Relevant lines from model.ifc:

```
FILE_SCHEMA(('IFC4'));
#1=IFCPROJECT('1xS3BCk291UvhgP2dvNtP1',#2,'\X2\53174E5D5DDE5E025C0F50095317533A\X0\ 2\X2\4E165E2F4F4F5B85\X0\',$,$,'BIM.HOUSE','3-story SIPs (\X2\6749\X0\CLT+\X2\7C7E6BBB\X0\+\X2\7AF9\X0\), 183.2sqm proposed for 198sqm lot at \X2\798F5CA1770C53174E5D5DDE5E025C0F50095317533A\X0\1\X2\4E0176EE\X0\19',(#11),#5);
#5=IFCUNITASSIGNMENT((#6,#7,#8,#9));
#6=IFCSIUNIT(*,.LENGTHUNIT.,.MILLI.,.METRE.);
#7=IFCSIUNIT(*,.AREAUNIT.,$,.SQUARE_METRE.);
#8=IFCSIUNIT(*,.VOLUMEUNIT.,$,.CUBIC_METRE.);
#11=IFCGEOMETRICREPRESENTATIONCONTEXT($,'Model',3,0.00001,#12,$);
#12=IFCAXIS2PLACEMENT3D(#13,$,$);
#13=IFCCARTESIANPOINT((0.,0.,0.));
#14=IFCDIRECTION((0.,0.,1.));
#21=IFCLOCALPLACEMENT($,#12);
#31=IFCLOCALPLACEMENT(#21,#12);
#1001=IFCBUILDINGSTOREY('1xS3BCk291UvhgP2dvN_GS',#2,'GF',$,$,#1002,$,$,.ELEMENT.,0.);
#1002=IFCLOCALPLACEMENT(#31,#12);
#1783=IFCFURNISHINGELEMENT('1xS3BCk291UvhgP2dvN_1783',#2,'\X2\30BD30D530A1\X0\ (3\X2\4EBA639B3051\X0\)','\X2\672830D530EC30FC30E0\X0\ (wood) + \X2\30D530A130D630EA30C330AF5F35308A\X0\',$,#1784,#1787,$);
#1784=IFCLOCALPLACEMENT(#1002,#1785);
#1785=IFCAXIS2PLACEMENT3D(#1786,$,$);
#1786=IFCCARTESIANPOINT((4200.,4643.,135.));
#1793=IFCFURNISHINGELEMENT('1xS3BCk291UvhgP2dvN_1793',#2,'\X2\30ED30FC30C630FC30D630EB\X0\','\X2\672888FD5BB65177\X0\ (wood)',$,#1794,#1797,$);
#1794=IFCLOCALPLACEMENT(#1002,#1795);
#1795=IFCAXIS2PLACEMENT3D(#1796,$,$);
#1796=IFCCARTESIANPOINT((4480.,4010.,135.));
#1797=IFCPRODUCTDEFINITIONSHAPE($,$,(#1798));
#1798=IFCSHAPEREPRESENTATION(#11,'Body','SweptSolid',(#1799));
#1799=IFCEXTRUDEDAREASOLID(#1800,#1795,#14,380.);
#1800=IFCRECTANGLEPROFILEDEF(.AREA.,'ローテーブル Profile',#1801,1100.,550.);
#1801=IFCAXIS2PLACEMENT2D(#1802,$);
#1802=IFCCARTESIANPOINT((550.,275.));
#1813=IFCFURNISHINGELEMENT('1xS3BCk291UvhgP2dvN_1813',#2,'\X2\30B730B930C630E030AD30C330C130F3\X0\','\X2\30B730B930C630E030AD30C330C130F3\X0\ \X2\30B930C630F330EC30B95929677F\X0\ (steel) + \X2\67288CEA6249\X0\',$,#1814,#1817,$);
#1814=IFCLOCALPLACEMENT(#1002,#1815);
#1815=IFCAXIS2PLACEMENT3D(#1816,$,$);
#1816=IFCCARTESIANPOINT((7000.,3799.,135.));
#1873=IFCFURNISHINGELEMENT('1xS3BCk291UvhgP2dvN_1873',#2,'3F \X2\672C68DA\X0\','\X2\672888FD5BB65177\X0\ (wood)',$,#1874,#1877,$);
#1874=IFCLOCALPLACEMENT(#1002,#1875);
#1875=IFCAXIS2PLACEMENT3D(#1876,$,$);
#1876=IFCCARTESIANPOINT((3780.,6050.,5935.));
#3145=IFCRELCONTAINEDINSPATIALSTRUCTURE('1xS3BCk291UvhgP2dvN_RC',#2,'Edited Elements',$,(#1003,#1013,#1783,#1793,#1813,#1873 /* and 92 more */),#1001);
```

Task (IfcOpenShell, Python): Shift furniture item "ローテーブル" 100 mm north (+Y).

```python
import ifcopenshell
import ifcopenshell.api.geometry
import ifcopenshell.util.placement
import ifcopenshell.util.unit

model = ifcopenshell.open("model.ifc")
unit_scale = ifcopenshell.util.unit.calculate_unit_scale(model)

item = model.by_guid("1xS3BCk291UvhgP2dvN_1793")
matrix = ifcopenshell.util.placement.get_local_placement(item.ObjectPlacement)
matrix[1, 3] += 0.1 / unit_scale
ifcopenshell.api.geometry.edit_object_placement(model, product=item, matrix=matrix, is_si=False)

print(ifcopenshell.util.placement.get_local_placement(item.ObjectPlacement).round(3) + 0.0)

model.write("model_rev.ifc")
```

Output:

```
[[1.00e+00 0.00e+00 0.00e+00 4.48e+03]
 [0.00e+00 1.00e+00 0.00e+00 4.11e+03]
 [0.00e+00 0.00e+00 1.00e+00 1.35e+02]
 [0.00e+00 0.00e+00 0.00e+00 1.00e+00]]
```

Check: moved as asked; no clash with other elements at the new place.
